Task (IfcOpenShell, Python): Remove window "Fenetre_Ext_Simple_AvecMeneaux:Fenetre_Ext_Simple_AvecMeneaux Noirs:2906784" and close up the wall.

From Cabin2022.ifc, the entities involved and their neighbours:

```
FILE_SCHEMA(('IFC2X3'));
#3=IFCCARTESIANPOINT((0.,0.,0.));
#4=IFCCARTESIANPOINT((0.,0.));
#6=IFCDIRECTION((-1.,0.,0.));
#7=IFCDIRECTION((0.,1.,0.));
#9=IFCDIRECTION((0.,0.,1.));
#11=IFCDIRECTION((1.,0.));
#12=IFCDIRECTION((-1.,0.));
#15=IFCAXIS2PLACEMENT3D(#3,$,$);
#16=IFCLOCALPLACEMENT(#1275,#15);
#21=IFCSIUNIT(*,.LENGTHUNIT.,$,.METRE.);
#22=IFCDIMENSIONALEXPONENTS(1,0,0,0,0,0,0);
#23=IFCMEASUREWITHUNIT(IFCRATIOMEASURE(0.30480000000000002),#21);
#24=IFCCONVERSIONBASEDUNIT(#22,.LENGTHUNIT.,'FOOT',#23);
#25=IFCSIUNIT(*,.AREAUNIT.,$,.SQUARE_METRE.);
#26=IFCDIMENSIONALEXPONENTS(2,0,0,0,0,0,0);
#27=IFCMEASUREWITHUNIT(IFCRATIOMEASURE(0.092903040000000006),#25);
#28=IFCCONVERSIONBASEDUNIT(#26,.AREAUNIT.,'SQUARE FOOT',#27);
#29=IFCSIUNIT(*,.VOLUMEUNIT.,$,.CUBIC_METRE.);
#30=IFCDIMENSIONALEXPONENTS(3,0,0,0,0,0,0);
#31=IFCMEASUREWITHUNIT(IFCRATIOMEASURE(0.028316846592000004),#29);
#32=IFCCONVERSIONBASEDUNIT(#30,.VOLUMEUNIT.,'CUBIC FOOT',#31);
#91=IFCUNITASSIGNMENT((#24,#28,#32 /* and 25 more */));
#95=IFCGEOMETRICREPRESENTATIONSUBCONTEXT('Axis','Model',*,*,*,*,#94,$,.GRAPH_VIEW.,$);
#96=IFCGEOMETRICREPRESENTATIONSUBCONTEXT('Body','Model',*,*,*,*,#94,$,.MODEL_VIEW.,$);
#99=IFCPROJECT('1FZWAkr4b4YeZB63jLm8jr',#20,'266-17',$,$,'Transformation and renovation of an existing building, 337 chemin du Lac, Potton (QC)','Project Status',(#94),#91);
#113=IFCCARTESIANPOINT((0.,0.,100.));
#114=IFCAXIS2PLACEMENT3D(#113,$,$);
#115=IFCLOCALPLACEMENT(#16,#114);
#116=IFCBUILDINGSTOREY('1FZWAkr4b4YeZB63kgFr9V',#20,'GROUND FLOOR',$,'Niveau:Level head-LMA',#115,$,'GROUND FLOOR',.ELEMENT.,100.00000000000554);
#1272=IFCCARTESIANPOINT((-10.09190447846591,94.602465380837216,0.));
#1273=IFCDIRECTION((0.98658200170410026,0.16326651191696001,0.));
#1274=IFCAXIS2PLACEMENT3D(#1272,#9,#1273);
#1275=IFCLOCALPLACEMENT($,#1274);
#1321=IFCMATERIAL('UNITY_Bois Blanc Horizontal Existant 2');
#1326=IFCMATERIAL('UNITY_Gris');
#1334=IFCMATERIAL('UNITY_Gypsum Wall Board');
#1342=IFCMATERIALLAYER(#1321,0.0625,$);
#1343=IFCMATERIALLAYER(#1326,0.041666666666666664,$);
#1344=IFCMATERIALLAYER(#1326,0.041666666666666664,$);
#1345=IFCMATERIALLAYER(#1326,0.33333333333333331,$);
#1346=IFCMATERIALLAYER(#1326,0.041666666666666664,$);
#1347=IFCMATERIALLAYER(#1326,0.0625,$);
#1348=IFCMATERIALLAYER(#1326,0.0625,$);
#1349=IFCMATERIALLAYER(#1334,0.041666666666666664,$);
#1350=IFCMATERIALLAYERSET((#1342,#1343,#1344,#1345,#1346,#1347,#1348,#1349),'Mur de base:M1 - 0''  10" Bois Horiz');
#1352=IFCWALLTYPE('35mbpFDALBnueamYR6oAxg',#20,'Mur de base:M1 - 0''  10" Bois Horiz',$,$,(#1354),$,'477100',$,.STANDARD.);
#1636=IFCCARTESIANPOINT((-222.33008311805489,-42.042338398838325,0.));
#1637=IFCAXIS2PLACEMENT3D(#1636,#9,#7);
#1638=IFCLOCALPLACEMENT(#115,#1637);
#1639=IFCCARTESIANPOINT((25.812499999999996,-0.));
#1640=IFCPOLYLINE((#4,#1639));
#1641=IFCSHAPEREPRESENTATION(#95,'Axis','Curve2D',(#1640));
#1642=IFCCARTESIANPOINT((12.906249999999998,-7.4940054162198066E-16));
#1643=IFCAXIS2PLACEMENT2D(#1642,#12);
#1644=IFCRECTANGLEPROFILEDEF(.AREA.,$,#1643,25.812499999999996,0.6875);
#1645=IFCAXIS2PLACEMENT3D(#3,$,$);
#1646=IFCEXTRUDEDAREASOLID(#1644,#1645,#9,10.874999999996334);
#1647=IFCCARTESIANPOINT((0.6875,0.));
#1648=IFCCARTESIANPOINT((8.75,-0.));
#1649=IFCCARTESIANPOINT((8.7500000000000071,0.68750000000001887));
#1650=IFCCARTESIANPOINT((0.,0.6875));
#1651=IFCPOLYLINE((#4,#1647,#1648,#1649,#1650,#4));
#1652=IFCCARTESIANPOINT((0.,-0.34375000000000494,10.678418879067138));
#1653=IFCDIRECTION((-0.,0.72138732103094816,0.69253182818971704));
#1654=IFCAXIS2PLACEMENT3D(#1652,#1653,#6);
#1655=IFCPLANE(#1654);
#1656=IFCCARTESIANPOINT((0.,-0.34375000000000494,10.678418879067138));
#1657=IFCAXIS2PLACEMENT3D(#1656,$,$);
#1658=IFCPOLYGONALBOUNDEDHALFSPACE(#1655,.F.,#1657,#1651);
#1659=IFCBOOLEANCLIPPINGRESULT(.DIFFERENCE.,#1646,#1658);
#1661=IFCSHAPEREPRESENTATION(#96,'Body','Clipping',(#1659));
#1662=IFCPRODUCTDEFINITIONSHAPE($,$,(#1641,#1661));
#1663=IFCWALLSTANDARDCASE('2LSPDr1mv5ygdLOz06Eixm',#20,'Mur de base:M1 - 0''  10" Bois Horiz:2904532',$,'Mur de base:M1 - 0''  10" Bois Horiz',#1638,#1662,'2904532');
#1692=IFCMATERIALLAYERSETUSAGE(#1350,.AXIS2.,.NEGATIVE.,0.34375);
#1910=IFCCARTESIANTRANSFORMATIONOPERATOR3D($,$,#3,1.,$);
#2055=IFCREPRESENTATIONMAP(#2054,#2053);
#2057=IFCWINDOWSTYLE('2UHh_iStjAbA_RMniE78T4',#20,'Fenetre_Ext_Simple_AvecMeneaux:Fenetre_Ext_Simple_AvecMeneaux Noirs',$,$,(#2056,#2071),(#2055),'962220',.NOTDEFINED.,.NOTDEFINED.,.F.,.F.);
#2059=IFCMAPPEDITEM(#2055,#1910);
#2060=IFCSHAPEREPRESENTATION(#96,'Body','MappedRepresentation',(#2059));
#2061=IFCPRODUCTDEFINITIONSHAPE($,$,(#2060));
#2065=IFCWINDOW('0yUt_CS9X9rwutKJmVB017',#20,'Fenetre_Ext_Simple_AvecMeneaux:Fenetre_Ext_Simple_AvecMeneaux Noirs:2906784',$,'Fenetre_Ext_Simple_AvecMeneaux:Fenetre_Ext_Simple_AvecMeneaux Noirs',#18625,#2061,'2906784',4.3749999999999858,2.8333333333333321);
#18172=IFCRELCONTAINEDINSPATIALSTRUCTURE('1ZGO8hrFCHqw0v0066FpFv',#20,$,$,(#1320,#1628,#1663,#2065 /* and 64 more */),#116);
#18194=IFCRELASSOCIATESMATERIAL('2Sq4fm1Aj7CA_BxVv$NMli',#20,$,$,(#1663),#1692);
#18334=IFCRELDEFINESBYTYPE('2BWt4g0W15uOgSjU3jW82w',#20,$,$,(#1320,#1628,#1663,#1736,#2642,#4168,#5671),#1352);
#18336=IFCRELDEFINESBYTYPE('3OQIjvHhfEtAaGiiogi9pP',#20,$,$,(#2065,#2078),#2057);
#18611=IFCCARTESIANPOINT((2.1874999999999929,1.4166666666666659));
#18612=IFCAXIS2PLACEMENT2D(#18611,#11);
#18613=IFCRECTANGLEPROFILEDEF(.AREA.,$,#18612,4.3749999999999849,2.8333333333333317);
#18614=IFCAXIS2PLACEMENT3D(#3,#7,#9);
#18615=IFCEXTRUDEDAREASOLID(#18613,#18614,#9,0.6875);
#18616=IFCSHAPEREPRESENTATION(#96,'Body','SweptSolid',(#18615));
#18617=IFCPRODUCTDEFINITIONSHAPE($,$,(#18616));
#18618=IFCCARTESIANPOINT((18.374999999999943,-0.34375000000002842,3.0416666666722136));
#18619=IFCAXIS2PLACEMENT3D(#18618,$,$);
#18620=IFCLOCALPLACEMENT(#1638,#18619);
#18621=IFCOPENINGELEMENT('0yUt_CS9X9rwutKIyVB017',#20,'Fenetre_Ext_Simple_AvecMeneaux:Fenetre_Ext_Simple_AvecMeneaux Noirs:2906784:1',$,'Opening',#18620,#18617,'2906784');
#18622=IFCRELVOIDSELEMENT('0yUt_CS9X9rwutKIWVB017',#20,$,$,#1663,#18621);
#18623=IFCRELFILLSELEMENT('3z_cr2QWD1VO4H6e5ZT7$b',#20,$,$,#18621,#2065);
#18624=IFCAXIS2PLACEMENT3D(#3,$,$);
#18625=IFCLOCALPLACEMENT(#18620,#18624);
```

```python
import ifcopenshell
import ifcopenshell.api.feature
import ifcopenshell.api.root
import ifcopenshell.geom
import ifcopenshell.util.shape

model = ifcopenshell.open("Cabin2022.ifc")
settings = ifcopenshell.geom.settings()


def volume(element):
    """Net volume in cubic metres, openings subtracted."""
    shape = ifcopenshell.geom.create_shape(settings, element)
    return ifcopenshell.util.shape.get_volume(shape.geometry)


window = model.by_guid("0yUt_CS9X9rwutKJmVB017")
opening = window.FillsVoids[0].RelatingOpeningElement
wall = opening.VoidsElements[0].RelatingBuildingElement
before = volume(wall)

ifcopenshell.api.root.remove_product(model, product=window)
ifcopenshell.api.feature.remove_feature(model, feature=opening)

after = volume(wall)

print(f"wall volume {before:.3f} -> {after:.3f} m3")

model.write("Cabin2022-out.ifc")
```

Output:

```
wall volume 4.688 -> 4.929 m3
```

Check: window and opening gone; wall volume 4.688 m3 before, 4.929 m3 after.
